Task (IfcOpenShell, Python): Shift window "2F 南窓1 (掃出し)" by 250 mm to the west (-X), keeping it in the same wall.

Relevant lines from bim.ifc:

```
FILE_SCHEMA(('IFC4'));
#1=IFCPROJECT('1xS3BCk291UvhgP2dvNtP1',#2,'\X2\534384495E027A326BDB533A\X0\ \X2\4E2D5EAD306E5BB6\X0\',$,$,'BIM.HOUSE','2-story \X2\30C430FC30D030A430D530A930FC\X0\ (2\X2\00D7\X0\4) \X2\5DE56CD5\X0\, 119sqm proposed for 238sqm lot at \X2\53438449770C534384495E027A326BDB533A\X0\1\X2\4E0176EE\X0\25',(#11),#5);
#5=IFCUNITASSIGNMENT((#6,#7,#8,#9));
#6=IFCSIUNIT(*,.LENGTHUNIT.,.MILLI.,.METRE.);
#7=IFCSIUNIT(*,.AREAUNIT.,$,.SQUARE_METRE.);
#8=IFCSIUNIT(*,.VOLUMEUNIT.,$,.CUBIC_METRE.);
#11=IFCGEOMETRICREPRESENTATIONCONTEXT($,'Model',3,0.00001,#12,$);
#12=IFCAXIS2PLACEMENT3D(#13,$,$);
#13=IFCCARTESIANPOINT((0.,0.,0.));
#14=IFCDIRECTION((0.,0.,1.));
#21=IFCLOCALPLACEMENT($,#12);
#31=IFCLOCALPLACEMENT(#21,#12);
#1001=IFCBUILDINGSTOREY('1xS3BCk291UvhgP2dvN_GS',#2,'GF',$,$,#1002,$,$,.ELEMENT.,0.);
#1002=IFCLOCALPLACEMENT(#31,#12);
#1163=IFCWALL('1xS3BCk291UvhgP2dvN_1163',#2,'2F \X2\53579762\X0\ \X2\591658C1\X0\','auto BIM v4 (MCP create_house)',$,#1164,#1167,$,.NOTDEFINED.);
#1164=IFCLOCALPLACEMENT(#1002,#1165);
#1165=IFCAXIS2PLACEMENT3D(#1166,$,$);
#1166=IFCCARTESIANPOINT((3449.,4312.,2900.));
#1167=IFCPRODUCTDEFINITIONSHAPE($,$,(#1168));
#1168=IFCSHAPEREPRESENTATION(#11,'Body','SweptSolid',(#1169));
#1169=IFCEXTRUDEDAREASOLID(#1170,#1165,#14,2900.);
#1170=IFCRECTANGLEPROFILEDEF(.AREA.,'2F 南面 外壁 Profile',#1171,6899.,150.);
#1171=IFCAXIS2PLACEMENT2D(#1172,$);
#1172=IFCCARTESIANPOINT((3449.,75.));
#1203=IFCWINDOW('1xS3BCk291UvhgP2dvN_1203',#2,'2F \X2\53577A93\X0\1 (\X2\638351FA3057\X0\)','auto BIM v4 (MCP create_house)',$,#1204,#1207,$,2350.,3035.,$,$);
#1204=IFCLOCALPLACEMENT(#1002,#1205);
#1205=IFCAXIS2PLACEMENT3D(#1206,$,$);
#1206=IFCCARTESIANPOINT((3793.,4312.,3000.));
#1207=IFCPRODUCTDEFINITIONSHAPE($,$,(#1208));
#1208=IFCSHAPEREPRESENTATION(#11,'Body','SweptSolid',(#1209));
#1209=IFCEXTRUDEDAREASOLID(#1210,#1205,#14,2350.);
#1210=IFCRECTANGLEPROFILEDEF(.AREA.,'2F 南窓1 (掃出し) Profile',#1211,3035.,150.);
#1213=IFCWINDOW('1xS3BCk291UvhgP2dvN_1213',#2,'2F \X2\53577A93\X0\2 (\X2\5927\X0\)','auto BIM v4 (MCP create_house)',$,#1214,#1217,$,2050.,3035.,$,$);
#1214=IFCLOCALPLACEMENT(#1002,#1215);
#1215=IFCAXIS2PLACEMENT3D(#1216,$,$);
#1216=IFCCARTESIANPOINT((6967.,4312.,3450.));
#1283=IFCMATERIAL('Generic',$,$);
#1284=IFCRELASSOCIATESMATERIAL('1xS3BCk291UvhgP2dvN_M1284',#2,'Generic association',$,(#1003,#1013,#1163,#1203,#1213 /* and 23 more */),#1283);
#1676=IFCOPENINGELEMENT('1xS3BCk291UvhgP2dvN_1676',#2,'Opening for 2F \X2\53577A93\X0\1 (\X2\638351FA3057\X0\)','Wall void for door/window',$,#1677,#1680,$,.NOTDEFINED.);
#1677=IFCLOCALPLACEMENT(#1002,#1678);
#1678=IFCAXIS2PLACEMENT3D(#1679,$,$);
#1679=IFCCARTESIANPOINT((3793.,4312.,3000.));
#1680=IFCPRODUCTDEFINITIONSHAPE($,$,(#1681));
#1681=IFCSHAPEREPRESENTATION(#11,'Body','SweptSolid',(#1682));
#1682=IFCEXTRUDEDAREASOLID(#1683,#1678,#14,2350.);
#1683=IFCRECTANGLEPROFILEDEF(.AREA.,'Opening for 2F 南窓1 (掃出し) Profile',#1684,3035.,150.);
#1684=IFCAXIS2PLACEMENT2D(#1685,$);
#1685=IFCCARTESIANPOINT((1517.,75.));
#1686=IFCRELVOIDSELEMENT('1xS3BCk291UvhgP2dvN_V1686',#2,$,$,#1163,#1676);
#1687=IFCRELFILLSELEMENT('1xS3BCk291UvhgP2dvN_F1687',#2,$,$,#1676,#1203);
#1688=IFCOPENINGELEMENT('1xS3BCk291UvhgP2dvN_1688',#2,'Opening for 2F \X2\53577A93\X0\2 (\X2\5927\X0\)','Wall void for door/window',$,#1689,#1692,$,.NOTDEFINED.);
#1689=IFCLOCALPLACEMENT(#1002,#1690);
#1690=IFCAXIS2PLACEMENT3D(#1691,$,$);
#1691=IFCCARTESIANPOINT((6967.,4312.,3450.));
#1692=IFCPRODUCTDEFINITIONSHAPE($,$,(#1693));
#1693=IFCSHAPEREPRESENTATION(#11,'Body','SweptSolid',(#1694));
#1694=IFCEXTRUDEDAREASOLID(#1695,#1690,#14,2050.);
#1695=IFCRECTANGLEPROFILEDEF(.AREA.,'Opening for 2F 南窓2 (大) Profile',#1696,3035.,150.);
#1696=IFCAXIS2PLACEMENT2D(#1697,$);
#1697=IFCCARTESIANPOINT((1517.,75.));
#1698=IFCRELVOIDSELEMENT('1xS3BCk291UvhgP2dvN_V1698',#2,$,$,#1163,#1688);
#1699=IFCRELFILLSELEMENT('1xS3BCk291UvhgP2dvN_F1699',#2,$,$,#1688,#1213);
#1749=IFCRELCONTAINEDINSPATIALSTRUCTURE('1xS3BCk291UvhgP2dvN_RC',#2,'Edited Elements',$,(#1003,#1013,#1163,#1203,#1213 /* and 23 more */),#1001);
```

```python
import ifcopenshell
import ifcopenshell.api.geometry
import ifcopenshell.util.placement
import ifcopenshell.util.unit

model = ifcopenshell.open("bim.ifc")
unit_scale = ifcopenshell.util.unit.calculate_unit_scale(model)

window = model.by_guid("1xS3BCk291UvhgP2dvN_1203")
opening = window.FillsVoids[0].RelatingOpeningElement
wall = opening.VoidsElements[0].RelatingBuildingElement

wall_matrix = ifcopenshell.util.placement.get_local_placement(wall.ObjectPlacement)
shift = wall_matrix[:3, 0] * -0.25 / unit_scale
before = ifcopenshell.util.placement.get_local_placement(window.ObjectPlacement)[:3, 3].copy()

# The window is not placed relative to its opening, so move both.
for product in (opening, window):
    matrix = ifcopenshell.util.placement.get_local_placement(product.ObjectPlacement)
    matrix[:3, 3] += shift
    ifcopenshell.api.geometry.edit_object_placement(model, product=product, matrix=matrix, is_si=False)

after = ifcopenshell.util.placement.get_local_placement(window.ObjectPlacement)[:3, 3]
print("window moved by", (after - before).round(3) + 0.0)

model.write("bim_edited.ifc")
```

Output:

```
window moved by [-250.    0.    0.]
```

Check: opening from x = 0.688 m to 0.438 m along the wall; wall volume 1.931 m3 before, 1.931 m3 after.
